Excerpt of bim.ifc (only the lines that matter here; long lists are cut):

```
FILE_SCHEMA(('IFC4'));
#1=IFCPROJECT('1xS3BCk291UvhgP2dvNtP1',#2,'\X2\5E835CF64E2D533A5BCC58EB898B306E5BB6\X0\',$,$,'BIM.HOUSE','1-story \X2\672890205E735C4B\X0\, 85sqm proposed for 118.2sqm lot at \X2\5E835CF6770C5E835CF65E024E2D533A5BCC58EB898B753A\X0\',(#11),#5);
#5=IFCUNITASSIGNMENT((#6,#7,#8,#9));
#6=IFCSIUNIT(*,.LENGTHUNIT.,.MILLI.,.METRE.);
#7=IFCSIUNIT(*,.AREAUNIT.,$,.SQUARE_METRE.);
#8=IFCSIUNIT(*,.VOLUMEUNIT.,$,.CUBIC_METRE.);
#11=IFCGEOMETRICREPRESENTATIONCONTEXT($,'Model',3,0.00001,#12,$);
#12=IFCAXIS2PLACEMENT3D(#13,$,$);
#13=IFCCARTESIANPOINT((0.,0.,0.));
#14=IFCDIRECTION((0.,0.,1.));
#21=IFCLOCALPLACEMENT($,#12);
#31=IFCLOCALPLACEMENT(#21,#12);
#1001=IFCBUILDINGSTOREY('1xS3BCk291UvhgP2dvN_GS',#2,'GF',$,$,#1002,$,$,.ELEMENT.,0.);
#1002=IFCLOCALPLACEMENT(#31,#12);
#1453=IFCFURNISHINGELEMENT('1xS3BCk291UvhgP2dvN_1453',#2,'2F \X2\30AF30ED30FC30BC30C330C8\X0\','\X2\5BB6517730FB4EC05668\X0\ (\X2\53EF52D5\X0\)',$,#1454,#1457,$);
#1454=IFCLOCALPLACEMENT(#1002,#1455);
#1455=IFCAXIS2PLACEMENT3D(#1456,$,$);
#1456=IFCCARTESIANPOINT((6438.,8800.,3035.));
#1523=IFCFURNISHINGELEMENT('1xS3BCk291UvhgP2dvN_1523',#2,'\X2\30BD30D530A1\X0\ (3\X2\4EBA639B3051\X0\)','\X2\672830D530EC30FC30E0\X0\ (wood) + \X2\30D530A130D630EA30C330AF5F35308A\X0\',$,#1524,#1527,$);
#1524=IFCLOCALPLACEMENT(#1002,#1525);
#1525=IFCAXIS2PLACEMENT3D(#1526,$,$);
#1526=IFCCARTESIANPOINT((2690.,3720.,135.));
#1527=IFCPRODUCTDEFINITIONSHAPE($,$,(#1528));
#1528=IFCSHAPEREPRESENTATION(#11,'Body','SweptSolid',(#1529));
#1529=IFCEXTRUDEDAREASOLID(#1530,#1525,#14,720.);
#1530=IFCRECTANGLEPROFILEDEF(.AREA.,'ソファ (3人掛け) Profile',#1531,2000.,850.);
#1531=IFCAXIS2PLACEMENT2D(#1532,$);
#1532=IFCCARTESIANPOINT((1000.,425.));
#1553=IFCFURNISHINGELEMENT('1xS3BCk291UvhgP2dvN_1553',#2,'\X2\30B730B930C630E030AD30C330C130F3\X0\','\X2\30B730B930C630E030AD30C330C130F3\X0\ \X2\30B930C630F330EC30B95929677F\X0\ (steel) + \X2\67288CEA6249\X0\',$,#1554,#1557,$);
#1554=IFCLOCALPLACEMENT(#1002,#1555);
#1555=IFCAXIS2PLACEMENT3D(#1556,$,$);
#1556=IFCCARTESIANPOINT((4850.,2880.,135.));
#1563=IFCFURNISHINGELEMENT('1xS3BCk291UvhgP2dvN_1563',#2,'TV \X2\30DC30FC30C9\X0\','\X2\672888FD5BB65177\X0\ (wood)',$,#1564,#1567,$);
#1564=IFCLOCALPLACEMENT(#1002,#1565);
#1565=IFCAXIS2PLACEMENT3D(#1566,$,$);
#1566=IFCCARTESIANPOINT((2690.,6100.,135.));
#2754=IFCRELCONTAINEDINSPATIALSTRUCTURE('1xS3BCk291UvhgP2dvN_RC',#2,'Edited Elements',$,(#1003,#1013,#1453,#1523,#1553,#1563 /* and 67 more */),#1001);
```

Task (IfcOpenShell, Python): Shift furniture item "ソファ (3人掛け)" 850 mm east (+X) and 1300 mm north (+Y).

```python
import ifcopenshell
import ifcopenshell.api.geometry
import ifcopenshell.util.placement
import ifcopenshell.util.unit

model = ifcopenshell.open("bim.ifc")
unit_scale = ifcopenshell.util.unit.calculate_unit_scale(model)

item = model.by_guid("1xS3BCk291UvhgP2dvN_1523")
matrix = ifcopenshell.util.placement.get_local_placement(item.ObjectPlacement)
matrix[0, 3] += 0.85 / unit_scale
matrix[1, 3] += 1.3 / unit_scale
ifcopenshell.api.geometry.edit_object_placement(model, product=item, matrix=matrix, is_si=False)

print(ifcopenshell.util.placement.get_local_placement(item.ObjectPlacement).round(3) + 0.0)

model.write("bim_v2.ifc")
```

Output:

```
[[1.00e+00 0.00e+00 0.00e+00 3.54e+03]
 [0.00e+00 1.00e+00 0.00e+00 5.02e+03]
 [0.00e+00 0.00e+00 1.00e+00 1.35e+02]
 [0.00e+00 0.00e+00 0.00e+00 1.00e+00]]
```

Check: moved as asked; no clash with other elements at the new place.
